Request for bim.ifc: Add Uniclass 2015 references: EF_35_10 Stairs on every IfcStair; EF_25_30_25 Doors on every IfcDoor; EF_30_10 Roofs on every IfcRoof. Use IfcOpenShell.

First a look at what the model holds.

```python
import ifcopenshell

model = ifcopenshell.open("bim.ifc")
print(model.schema)
print("classifications:", [c.Name for c in model.by_type("IfcClassification")])
for ifc_class in ("IfcDoor", "IfcRoof", "IfcStair", "IfcWall", "IfcWindow"):
    print(ifc_class, len(model.by_type(ifc_class)))
```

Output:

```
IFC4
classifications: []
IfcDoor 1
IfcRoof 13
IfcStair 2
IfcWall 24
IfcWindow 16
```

```python
import ifcopenshell
import ifcopenshell.api.classification

model = ifcopenshell.open("bim.ifc")

system = ifcopenshell.api.classification.add_classification(model, classification="Uniclass 2015")

codes = {
    "IfcStair": ("EF_35_10", "Stairs"),
    "IfcDoor": ("EF_25_30_25", "Doors"),
    "IfcRoof": ("EF_30_10", "Roofs"),
}
for ifc_class, (code, name) in codes.items():
    products = model.by_type(ifc_class)
    ifcopenshell.api.classification.add_reference(
        model, products=products, classification=system, identification=code, name=name
    )
    print(code, len(products))

model.write("bim-out.ifc")
```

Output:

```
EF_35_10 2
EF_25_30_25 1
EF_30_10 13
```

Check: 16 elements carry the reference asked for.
